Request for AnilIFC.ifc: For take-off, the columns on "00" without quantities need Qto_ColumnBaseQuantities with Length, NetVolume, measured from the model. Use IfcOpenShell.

First a look at what the model holds.

```python
import ifcopenshell
import ifcopenshell.util.element
import ifcopenshell.util.unit

model = ifcopenshell.open("AnilIFC.ifc")
print(model.schema)
for unit_type in ("LENGTHUNIT", "AREAUNIT", "VOLUMEUNIT"):
    print(unit_type, ifcopenshell.util.unit.calculate_unit_scale(model, unit_type))
storey = next(s for s in model.by_type("IfcBuildingStorey") if s.Name == "00")
columns = [e for e in ifcopenshell.util.element.get_decomposition(storey) if e.is_a("IfcColumn")]
for e in sorted(columns, key=lambda e: e.id()):
    print(e.id(), e.is_a(), e.Name, list(ifcopenshell.util.element.get_psets(e, qtos_only=True)), sep=" | ")
```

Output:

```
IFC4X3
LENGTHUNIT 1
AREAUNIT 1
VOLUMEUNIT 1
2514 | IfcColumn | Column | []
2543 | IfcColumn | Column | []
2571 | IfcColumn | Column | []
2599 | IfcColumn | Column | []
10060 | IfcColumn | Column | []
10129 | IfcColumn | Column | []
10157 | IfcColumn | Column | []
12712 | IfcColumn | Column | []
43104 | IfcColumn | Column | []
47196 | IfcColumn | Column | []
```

```python
import ifcopenshell
import ifcopenshell.api.pset
import ifcopenshell.geom
import ifcopenshell.util.element
import ifcopenshell.util.shape
import ifcopenshell.util.unit

model = ifcopenshell.open("AnilIFC.ifc")
unit_scale = ifcopenshell.util.unit.calculate_unit_scale(model)
volume_scale = ifcopenshell.util.unit.calculate_unit_scale(model, "VOLUMEUNIT")
settings = ifcopenshell.geom.settings()

storey = next(s for s in model.by_type("IfcBuildingStorey") if s.Name == "00")
columns = [e for e in ifcopenshell.util.element.get_decomposition(storey) if e.is_a("IfcColumn")]

for e in sorted(columns, key=lambda e: e.id()):
    if ifcopenshell.util.element.get_psets(e, qtos_only=True, should_inherit=False):
        continue
    # Geometry comes back in metres, in the element's own axes.
    shape = ifcopenshell.geom.create_shape(settings, e)
    values = {
        "Length": ifcopenshell.util.shape.get_z(shape.geometry) / unit_scale,
        "NetVolume": ifcopenshell.util.shape.get_volume(shape.geometry) / volume_scale,
    }
    qto = ifcopenshell.api.pset.add_qto(model, product=e, name="Qto_ColumnBaseQuantities")
    ifcopenshell.api.pset.edit_qto(model, qto=qto, properties=values)
    print(e.id(), {k: round(v, 3) for k, v in values.items()})

model.write("AnilIFC_v2.ifc")
```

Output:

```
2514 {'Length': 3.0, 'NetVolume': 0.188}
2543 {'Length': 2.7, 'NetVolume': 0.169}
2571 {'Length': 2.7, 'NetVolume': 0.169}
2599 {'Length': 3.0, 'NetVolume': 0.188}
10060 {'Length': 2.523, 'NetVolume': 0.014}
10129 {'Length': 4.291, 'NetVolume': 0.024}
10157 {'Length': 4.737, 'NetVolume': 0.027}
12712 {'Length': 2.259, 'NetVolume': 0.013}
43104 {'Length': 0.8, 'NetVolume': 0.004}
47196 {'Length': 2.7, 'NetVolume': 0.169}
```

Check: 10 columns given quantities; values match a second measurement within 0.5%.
